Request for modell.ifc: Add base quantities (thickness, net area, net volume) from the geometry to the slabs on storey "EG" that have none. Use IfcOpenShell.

First a look at what the model holds.

```python
import ifcopenshell
import ifcopenshell.util.element
import ifcopenshell.util.unit

model = ifcopenshell.open("modell.ifc")
print(model.schema)
for unit_type in ("LENGTHUNIT", "AREAUNIT", "VOLUMEUNIT"):
    print(unit_type, ifcopenshell.util.unit.calculate_unit_scale(model, unit_type))
storey = next(s for s in model.by_type("IfcBuildingStorey") if s.Name == "EG")
slabs = [e for e in ifcopenshell.util.element.get_decomposition(storey) if e.is_a("IfcSlab")]
for e in sorted(slabs, key=lambda e: e.id()):
    print(e.id(), e.is_a(), e.Name, list(ifcopenshell.util.element.get_psets(e, qtos_only=True)), sep=" | ")
```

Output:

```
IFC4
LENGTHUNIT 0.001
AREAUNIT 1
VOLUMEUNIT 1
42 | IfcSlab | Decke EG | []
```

```python
import ifcopenshell
import ifcopenshell.api.pset
import ifcopenshell.geom
import ifcopenshell.util.element
import ifcopenshell.util.shape
import ifcopenshell.util.unit

model = ifcopenshell.open("modell.ifc")
unit_scale = ifcopenshell.util.unit.calculate_unit_scale(model)
area_scale = ifcopenshell.util.unit.calculate_unit_scale(model, "AREAUNIT")
volume_scale = ifcopenshell.util.unit.calculate_unit_scale(model, "VOLUMEUNIT")
settings = ifcopenshell.geom.settings()

storey = next(s for s in model.by_type("IfcBuildingStorey") if s.Name == "EG")
slabs = [e for e in ifcopenshell.util.element.get_decomposition(storey) if e.is_a("IfcSlab")]

for e in sorted(slabs, key=lambda e: e.id()):
    if ifcopenshell.util.element.get_psets(e, qtos_only=True, should_inherit=False):
        continue
    # Geometry comes back in metres, in the element's own axes.
    shape = ifcopenshell.geom.create_shape(settings, e)
    values = {
        "Width": ifcopenshell.util.shape.get_z(shape.geometry) / unit_scale,
        "NetArea": ifcopenshell.util.shape.get_footprint_area(shape.geometry) / area_scale,
        "NetVolume": ifcopenshell.util.shape.get_volume(shape.geometry) / volume_scale,
    }
    qto = ifcopenshell.api.pset.add_qto(model, product=e, name="Qto_SlabBaseQuantities")
    ifcopenshell.api.pset.edit_qto(model, qto=qto, properties=values)
    print(e.id(), {k: round(v, 3) for k, v in values.items()})

model.write("modell_v2.ifc")
```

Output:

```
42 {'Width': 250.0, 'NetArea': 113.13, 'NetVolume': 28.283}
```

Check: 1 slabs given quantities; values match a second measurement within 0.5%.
